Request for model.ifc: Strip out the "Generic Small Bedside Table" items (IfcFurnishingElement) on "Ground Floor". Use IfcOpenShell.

First a look at what the model holds.

```python
import ifcopenshell
import ifcopenshell.util.element

model = ifcopenshell.open("model.ifc")
print(model.schema)
storey = next(s for s in model.by_type("IfcBuildingStorey") if s.Name == "Ground Floor")
furniture = [e for e in ifcopenshell.util.element.get_decomposition(storey) if e.is_a("IfcFurnishingElement")]
seen = {}
for e in furniture:
    element_type = ifcopenshell.util.element.get_type(e)
    name = element_type.Name if element_type not in (None, e) else None
    seen[name] = seen.get(name, 0) + 1
for name, count in sorted(seen.items(), key=str):
    print(count, "x", name)
```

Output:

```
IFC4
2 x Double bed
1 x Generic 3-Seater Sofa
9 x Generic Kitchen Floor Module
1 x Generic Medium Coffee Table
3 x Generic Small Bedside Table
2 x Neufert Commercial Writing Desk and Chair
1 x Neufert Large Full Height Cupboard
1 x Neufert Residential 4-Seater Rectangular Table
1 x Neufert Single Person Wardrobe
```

```python
import ifcopenshell
import ifcopenshell.api.root
import ifcopenshell.util.element

model = ifcopenshell.open("model.ifc")

storey = next(s for s in model.by_type("IfcBuildingStorey") if s.Name == "Ground Floor")
furniture = [e for e in ifcopenshell.util.element.get_decomposition(storey) if e.is_a("IfcFurnishingElement")]
targets = [e for e in furniture if (t := ifcopenshell.util.element.get_type(e)) not in (None, e) and t.Name == "Generic Small Bedside Table"]

for e in targets:
    ifcopenshell.api.root.remove_product(model, product=e)
print(len(targets), "removed")

model.write("model_updated.ifc")
```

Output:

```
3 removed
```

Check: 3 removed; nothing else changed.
